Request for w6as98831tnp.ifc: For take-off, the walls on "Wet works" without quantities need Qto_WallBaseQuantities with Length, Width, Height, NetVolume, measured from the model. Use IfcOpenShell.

First a look at what the model holds.

```python
import ifcopenshell
import ifcopenshell.util.element
import ifcopenshell.util.unit

model = ifcopenshell.open("w6as98831tnp.ifc")
print(model.schema)
for unit_type in ("LENGTHUNIT", "AREAUNIT", "VOLUMEUNIT"):
    print(unit_type, ifcopenshell.util.unit.calculate_unit_scale(model, unit_type))
storey = next(s for s in model.by_type("IfcBuildingStorey") if s.Name == "Wet works")
walls = [e for e in ifcopenshell.util.element.get_decomposition(storey) if e.is_a("IfcWall")]
for e in sorted(walls, key=lambda e: e.id()):
    print(e.id(), e.is_a(), e.Name, list(ifcopenshell.util.element.get_psets(e, qtos_only=True)), sep=" | ")
```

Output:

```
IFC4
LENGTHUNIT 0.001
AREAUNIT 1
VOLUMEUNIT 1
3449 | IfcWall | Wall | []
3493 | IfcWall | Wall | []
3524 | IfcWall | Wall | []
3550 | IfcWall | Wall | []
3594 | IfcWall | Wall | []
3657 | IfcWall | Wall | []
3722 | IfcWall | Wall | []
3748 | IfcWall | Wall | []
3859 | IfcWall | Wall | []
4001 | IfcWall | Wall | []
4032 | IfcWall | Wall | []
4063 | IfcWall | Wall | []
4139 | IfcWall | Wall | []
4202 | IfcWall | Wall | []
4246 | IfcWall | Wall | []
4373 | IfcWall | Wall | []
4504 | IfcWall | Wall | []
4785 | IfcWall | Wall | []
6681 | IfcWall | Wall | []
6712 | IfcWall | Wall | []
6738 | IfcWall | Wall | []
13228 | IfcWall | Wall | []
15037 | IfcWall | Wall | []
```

```python
import ifcopenshell
import ifcopenshell.api.pset
import ifcopenshell.geom
import ifcopenshell.util.element
import ifcopenshell.util.shape
import ifcopenshell.util.unit

model = ifcopenshell.open("w6as98831tnp.ifc")
unit_scale = ifcopenshell.util.unit.calculate_unit_scale(model)
volume_scale = ifcopenshell.util.unit.calculate_unit_scale(model, "VOLUMEUNIT")
settings = ifcopenshell.geom.settings()

storey = next(s for s in model.by_type("IfcBuildingStorey") if s.Name == "Wet works")
walls = [e for e in ifcopenshell.util.element.get_decomposition(storey) if e.is_a("IfcWall")]

for e in sorted(walls, key=lambda e: e.id()):
    if ifcopenshell.util.element.get_psets(e, qtos_only=True, should_inherit=False):
        continue
    # Geometry comes back in metres, in the element's own axes.
    shape = ifcopenshell.geom.create_shape(settings, e)
    values = {
        "Length": ifcopenshell.util.shape.get_x(shape.geometry) / unit_scale,
        "Width": ifcopenshell.util.shape.get_y(shape.geometry) / unit_scale,
        "Height": ifcopenshell.util.shape.get_z(shape.geometry) / unit_scale,
        "NetVolume": ifcopenshell.util.shape.get_volume(shape.geometry) / volume_scale,
    }
    qto = ifcopenshell.api.pset.add_qto(model, product=e, name="Qto_WallBaseQuantities")
    ifcopenshell.api.pset.edit_qto(model, qto=qto, properties=values)
    print(e.id(), {k: round(v, 3) for k, v in values.items()})

model.write("w6as98831tnp_edited.ifc")
```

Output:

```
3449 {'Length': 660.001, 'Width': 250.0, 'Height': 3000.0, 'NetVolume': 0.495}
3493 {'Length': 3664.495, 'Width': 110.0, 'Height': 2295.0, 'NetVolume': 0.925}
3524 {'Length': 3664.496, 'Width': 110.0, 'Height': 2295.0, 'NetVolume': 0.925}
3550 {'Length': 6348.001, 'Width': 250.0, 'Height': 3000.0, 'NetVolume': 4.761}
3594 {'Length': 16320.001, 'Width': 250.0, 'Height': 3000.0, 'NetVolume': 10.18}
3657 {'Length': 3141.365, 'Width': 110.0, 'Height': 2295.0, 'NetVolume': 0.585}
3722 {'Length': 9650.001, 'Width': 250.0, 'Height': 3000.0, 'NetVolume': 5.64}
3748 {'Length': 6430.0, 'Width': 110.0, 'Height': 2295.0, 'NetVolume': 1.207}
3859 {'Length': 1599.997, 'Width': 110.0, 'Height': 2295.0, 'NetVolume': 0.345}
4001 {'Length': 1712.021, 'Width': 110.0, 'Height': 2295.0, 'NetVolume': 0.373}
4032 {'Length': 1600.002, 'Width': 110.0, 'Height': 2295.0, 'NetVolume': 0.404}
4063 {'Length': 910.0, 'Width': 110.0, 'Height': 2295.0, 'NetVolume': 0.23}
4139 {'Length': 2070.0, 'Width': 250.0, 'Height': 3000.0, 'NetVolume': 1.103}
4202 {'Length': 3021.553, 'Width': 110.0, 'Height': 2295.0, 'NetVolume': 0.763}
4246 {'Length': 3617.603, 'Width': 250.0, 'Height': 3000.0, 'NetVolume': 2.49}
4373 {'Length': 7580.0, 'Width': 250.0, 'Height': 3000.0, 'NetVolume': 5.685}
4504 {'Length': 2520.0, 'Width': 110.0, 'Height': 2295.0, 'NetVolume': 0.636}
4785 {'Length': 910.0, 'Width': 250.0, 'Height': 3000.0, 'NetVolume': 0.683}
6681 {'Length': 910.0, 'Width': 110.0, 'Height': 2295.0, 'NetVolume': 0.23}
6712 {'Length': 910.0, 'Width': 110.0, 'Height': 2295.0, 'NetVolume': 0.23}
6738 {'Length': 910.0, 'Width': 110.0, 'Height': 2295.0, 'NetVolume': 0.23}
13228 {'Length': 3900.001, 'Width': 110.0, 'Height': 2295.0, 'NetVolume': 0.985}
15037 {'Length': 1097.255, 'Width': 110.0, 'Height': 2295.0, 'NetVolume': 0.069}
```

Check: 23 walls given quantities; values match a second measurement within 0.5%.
